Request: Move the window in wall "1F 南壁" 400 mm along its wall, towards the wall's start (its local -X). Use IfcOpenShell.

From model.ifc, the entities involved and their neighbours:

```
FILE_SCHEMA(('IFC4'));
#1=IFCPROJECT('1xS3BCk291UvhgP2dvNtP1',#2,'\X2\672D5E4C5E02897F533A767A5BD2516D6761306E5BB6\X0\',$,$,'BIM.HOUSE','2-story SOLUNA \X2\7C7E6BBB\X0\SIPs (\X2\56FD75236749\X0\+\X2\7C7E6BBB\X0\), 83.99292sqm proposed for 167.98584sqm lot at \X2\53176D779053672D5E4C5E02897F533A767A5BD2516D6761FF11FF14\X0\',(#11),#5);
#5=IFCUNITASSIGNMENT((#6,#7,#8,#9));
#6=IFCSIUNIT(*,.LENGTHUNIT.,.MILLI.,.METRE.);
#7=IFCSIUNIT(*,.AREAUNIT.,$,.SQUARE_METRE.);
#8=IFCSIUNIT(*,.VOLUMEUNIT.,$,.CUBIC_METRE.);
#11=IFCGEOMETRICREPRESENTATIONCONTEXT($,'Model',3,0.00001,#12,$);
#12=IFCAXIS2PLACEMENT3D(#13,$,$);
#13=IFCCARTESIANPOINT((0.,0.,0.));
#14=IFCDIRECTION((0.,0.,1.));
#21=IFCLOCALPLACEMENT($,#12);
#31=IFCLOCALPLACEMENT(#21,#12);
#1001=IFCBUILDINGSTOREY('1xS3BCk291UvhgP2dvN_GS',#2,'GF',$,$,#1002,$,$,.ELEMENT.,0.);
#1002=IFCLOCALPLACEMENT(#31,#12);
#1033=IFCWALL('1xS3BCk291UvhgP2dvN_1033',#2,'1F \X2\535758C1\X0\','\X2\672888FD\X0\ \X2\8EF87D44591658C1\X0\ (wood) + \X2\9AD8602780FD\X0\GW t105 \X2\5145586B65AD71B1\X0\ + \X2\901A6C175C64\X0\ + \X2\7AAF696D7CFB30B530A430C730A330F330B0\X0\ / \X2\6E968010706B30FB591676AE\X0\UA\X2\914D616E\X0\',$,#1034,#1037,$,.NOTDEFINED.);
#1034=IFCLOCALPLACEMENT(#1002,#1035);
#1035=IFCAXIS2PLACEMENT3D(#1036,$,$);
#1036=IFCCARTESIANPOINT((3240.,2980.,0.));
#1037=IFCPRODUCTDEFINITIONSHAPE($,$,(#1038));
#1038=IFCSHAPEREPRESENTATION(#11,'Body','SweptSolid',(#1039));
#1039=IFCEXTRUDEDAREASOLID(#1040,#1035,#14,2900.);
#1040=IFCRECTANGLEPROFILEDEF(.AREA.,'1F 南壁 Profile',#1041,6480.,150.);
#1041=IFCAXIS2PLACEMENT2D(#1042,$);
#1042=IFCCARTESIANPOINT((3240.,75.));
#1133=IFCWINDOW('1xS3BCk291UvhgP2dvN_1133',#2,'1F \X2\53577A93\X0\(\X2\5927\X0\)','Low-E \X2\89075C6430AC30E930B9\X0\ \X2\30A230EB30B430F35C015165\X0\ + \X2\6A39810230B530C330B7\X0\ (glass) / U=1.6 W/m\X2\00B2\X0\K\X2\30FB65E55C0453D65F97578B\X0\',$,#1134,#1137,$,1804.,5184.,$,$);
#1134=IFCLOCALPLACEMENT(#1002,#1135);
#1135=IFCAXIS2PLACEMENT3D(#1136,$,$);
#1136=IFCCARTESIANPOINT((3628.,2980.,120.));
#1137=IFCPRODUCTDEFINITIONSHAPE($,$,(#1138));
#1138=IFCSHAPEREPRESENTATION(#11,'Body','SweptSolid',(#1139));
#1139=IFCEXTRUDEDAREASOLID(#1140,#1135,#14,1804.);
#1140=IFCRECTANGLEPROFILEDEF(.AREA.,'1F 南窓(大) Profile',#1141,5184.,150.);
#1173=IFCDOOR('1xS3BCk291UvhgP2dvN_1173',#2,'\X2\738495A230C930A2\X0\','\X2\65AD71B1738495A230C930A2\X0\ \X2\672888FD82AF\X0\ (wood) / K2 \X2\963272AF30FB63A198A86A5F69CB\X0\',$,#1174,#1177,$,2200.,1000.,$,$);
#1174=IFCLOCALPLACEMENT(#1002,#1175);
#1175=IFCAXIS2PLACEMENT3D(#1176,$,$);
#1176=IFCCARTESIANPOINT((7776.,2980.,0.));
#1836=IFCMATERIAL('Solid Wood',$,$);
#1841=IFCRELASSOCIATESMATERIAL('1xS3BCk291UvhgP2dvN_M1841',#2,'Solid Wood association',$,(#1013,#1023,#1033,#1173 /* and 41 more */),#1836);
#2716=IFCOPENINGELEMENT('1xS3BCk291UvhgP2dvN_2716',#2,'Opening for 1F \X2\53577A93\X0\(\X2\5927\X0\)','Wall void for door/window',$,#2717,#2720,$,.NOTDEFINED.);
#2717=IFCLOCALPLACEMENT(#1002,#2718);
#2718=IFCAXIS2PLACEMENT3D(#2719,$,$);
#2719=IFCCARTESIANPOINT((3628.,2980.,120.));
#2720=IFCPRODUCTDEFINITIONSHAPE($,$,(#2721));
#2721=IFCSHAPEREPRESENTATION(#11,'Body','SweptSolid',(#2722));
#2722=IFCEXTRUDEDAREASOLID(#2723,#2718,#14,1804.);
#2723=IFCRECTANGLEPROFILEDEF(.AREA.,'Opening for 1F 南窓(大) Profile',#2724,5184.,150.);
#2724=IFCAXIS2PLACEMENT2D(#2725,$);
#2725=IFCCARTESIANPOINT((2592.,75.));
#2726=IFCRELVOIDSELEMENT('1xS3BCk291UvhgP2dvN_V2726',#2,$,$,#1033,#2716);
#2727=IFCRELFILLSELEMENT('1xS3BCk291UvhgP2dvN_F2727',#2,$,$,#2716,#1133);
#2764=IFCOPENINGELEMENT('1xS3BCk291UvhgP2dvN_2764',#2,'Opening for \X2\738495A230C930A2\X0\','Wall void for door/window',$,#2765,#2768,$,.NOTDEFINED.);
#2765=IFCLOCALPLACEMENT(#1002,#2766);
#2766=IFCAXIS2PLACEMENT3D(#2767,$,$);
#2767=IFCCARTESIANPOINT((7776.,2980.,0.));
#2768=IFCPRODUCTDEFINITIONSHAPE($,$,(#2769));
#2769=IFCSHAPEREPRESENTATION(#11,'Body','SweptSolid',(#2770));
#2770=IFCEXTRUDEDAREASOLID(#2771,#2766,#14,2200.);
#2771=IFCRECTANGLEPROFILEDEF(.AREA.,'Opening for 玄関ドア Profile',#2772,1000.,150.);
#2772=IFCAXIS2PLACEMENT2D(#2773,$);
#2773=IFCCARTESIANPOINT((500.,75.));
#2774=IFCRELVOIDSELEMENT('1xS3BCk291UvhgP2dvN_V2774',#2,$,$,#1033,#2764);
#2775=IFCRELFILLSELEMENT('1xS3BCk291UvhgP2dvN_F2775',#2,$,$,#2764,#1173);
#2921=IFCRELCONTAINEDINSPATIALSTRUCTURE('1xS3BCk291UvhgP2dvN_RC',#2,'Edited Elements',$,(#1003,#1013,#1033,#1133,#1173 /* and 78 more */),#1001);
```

```python
import ifcopenshell
import ifcopenshell.api.geometry
import ifcopenshell.util.placement
import ifcopenshell.util.unit

model = ifcopenshell.open("model.ifc")
unit_scale = ifcopenshell.util.unit.calculate_unit_scale(model)

window = model.by_id(1133)
opening = window.FillsVoids[0].RelatingOpeningElement
wall = opening.VoidsElements[0].RelatingBuildingElement

wall_matrix = ifcopenshell.util.placement.get_local_placement(wall.ObjectPlacement)
shift = wall_matrix[:3, 0] * -0.4 / unit_scale
before = ifcopenshell.util.placement.get_local_placement(window.ObjectPlacement)[:3, 3].copy()

# The window is not placed relative to its opening, so move both.
for product in (opening, window):
    matrix = ifcopenshell.util.placement.get_local_placement(product.ObjectPlacement)
    matrix[:3, 3] += shift
    ifcopenshell.api.geometry.edit_object_placement(model, product=product, matrix=matrix, is_si=False)

after = ifcopenshell.util.placement.get_local_placement(window.ObjectPlacement)[:3, 3]
print("window moved by", (after - before).round(3) + 0.0)

model.write("model_rev.ifc")
```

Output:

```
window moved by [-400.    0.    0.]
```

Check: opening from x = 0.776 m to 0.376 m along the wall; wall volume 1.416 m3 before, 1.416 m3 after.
